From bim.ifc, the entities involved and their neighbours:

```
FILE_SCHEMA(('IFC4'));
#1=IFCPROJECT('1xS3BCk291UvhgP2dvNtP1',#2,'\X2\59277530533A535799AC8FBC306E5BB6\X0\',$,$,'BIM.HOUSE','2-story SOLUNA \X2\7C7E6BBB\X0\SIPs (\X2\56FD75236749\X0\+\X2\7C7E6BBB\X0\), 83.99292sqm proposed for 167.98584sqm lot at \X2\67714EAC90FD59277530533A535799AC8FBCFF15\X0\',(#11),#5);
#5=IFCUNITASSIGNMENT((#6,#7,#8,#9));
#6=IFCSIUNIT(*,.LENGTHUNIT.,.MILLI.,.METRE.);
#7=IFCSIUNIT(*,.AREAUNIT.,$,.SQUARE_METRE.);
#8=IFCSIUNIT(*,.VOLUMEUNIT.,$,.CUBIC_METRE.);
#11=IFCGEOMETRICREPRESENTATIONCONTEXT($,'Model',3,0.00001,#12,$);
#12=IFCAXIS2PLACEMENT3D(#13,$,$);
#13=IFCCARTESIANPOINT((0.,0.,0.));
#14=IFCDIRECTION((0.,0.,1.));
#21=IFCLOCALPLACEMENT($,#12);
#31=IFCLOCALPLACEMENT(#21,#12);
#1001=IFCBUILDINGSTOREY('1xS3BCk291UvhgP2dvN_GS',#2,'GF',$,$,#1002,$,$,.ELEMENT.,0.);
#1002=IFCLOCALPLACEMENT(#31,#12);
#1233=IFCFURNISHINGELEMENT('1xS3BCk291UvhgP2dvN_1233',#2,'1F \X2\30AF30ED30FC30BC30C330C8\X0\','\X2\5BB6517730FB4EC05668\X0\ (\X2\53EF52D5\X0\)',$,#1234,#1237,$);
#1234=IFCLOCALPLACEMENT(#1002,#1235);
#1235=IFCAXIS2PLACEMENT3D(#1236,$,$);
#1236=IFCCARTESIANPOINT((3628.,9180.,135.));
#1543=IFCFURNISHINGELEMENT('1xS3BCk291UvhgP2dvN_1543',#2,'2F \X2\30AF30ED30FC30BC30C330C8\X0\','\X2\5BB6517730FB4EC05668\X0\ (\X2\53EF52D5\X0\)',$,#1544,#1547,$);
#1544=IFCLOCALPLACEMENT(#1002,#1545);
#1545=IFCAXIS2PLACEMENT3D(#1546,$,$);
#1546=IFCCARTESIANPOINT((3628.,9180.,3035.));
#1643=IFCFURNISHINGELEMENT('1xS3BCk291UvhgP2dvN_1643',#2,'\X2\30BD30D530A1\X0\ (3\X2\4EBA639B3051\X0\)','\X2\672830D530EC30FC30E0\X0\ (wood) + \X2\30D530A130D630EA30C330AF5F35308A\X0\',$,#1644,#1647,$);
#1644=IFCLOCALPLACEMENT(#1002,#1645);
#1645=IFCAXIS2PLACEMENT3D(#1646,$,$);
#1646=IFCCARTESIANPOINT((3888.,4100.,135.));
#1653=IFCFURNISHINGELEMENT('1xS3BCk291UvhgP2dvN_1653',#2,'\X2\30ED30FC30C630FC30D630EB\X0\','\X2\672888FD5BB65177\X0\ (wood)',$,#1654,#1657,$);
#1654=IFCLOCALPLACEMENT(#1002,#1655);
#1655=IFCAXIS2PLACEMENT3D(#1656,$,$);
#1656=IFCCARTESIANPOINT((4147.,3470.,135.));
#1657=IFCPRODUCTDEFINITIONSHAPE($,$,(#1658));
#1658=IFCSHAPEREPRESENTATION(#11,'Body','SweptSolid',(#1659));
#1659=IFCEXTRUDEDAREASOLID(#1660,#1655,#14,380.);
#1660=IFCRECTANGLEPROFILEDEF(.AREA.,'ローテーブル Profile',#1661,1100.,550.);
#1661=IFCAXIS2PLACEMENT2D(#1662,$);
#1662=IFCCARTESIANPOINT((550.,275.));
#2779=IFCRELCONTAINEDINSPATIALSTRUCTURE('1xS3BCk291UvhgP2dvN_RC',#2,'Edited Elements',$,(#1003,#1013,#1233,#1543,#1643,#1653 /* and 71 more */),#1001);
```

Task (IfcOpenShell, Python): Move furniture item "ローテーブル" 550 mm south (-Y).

```python
import ifcopenshell
import ifcopenshell.api.geometry
import ifcopenshell.util.placement
import ifcopenshell.util.unit

model = ifcopenshell.open("bim.ifc")
unit_scale = ifcopenshell.util.unit.calculate_unit_scale(model)

item = model.by_guid("1xS3BCk291UvhgP2dvN_1653")
matrix = ifcopenshell.util.placement.get_local_placement(item.ObjectPlacement)
matrix[1, 3] -= 0.55 / unit_scale
ifcopenshell.api.geometry.edit_object_placement(model, product=item, matrix=matrix, is_si=False)

print(ifcopenshell.util.placement.get_local_placement(item.ObjectPlacement).round(3) + 0.0)

model.write("bim-out.ifc")
```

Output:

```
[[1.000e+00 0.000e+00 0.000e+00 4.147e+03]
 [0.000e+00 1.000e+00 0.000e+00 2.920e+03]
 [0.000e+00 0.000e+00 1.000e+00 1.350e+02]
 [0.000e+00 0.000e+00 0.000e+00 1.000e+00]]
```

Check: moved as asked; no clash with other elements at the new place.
